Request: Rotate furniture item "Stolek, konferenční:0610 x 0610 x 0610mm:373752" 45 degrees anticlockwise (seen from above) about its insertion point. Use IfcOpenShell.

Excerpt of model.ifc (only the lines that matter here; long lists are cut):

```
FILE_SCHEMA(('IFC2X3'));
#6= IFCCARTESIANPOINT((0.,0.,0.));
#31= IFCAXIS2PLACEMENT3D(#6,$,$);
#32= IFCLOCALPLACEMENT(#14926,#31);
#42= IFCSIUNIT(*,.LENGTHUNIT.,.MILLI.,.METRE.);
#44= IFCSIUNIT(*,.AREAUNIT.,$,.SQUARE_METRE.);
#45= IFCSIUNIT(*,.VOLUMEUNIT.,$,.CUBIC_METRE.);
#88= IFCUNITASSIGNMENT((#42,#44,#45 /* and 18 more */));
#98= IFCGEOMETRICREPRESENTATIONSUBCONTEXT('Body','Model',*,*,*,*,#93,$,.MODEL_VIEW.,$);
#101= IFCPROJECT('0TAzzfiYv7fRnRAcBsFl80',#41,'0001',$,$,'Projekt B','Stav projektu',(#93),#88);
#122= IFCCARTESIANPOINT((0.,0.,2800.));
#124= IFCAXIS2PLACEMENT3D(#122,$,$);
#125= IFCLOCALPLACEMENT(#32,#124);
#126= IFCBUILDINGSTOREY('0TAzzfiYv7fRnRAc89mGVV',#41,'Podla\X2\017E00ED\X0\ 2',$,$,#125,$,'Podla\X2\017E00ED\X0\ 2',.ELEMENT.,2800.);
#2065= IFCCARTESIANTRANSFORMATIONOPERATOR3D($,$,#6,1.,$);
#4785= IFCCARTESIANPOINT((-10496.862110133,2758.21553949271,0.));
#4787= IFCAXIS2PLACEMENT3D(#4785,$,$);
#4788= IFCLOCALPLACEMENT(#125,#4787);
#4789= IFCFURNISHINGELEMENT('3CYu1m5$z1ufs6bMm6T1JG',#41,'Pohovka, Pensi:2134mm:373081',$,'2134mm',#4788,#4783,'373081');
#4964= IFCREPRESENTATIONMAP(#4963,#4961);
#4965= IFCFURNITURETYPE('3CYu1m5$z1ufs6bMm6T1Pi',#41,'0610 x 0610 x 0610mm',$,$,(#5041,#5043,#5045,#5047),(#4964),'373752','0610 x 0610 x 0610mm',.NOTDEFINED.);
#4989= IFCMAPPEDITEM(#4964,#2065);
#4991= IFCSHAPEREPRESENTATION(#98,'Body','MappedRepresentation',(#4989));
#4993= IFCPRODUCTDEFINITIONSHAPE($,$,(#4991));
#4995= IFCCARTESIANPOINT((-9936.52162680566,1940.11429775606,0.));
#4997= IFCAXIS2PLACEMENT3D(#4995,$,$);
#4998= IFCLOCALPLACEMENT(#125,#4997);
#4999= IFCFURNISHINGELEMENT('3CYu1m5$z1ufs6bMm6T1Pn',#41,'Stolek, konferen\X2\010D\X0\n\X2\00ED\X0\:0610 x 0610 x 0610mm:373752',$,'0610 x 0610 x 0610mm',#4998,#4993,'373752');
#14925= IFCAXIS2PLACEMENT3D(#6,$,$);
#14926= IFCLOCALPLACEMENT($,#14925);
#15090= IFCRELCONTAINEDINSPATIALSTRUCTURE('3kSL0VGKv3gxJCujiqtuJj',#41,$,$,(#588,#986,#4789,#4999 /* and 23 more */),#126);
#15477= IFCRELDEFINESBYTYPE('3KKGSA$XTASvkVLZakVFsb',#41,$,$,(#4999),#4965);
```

```python
import ifcopenshell
import ifcopenshell.api.geometry
import ifcopenshell.util.placement

model = ifcopenshell.open("model.ifc")

item = model.by_guid("3CYu1m5$z1ufs6bMm6T1Pn")
matrix = ifcopenshell.util.placement.get_local_placement(item.ObjectPlacement)
matrix = matrix @ ifcopenshell.util.placement.rotation(45, "Z")
ifcopenshell.api.geometry.edit_object_placement(model, product=item, matrix=matrix, is_si=False)

print(ifcopenshell.util.placement.get_local_placement(item.ObjectPlacement).round(3) + 0.0)

model.write("model_edited.ifc")
```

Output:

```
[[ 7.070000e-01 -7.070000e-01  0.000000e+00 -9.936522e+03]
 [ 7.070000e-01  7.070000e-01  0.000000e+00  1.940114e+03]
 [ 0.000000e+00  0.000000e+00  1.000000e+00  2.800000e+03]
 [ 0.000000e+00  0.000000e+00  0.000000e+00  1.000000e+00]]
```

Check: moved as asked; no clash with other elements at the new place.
